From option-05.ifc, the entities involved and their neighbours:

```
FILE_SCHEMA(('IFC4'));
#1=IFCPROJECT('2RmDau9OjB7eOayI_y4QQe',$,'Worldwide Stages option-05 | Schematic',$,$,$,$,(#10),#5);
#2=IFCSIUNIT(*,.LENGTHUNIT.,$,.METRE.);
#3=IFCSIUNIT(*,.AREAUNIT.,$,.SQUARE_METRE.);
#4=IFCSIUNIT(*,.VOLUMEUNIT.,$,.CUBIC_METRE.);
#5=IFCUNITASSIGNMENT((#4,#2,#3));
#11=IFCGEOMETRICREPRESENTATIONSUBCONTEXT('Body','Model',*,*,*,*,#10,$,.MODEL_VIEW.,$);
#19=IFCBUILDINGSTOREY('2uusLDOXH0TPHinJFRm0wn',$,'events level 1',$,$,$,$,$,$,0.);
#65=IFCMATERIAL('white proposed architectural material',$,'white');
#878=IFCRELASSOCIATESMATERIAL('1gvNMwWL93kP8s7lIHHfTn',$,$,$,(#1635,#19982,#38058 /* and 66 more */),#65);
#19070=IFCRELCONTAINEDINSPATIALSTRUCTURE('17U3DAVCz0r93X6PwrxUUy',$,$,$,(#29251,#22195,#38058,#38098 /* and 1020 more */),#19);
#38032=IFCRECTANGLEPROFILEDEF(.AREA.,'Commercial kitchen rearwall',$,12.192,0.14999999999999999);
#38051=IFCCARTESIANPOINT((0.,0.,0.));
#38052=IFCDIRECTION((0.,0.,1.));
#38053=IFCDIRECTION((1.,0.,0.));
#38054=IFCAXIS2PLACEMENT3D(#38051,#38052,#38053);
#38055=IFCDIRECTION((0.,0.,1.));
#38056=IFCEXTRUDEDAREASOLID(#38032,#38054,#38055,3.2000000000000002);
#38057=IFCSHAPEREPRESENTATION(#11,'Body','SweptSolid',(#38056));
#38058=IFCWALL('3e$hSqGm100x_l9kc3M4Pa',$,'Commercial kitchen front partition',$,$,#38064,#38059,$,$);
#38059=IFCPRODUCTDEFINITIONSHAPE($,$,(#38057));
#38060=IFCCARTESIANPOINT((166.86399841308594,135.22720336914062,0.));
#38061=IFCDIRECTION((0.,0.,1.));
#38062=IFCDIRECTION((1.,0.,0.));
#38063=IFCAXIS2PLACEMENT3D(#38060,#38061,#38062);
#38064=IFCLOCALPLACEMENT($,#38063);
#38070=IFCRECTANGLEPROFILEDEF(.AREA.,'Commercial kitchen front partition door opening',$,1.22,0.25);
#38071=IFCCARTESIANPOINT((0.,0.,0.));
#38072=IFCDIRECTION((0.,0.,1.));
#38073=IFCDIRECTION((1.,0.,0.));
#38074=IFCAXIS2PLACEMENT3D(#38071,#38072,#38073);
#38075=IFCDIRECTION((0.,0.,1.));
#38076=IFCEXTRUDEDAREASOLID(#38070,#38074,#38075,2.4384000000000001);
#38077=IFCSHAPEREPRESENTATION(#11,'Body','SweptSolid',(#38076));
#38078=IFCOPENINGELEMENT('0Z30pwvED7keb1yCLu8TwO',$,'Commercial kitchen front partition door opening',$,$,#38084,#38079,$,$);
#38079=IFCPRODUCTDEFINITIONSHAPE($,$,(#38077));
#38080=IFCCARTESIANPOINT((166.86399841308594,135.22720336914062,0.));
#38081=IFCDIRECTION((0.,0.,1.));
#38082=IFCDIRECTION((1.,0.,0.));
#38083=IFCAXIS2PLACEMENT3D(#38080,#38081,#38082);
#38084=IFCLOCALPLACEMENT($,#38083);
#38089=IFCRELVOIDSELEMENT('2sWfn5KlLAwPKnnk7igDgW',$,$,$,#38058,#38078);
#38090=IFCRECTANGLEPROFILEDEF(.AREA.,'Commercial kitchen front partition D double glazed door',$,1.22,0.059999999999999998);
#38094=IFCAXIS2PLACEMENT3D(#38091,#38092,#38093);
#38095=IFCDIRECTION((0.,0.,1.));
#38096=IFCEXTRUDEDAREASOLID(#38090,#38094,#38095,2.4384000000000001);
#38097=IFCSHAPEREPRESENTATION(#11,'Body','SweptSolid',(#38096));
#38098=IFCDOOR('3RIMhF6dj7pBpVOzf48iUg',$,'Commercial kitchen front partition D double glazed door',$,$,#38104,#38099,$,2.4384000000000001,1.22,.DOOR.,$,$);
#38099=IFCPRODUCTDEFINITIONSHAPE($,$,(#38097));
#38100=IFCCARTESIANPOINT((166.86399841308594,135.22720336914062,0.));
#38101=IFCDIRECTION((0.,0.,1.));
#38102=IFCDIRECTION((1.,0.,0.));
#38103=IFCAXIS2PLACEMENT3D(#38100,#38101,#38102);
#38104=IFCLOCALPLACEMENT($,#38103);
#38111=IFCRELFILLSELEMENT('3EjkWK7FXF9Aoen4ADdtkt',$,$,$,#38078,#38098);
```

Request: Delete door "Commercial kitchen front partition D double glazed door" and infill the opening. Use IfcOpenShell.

```python
import ifcopenshell
import ifcopenshell.api.feature
import ifcopenshell.api.root
import ifcopenshell.geom
import ifcopenshell.util.shape

model = ifcopenshell.open("option-05.ifc")
settings = ifcopenshell.geom.settings()


def volume(element):
    """Net volume in cubic metres, openings subtracted."""
    shape = ifcopenshell.geom.create_shape(settings, element)
    return ifcopenshell.util.shape.get_volume(shape.geometry)


door = model.by_guid("3RIMhF6dj7pBpVOzf48iUg")
opening = door.FillsVoids[0].RelatingOpeningElement
wall = opening.VoidsElements[0].RelatingBuildingElement
before = volume(wall)

ifcopenshell.api.root.remove_product(model, product=door)
ifcopenshell.api.feature.remove_feature(model, feature=opening)

after = volume(wall)

print(f"wall volume {before:.3f} -> {after:.3f} m3")

model.write("option-05-out.ifc")
```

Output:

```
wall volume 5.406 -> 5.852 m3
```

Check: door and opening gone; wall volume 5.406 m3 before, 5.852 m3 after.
